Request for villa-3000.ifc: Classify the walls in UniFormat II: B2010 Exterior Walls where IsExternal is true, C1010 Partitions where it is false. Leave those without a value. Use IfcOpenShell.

First a look at what the model holds.

```python
import ifcopenshell
import ifcopenshell.util.element

model = ifcopenshell.open("villa-3000.ifc")
print(model.schema)
print("classifications:", [c.Name for c in model.by_type("IfcClassification")])
values = [ifcopenshell.util.element.get_pset(e, "Pset_WallCommon", "IsExternal") for e in model.by_type("IfcWall")]
for value in (True, False, None):
    print("IsExternal", value, values.count(value))
```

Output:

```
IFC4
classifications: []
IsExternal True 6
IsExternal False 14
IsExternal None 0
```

```python
import ifcopenshell
import ifcopenshell.api.classification
import ifcopenshell.util.element

model = ifcopenshell.open("villa-3000.ifc")

system = ifcopenshell.api.classification.add_classification(model, classification="UniFormat II")

walls = model.by_type("IfcWall")
external = {e: ifcopenshell.util.element.get_pset(e, "Pset_WallCommon", "IsExternal") for e in walls}
for flag, code, name in ((True, "B2010", "Exterior Walls"), (False, "C1010", "Partitions")):
    products = [e for e in walls if external[e] is flag]
    ifcopenshell.api.classification.add_reference(
        model, products=products, classification=system, identification=code, name=name
    )
    print(code, len(products))

model.write("villa-3000_edited.ifc")
```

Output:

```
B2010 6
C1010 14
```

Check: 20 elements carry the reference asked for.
